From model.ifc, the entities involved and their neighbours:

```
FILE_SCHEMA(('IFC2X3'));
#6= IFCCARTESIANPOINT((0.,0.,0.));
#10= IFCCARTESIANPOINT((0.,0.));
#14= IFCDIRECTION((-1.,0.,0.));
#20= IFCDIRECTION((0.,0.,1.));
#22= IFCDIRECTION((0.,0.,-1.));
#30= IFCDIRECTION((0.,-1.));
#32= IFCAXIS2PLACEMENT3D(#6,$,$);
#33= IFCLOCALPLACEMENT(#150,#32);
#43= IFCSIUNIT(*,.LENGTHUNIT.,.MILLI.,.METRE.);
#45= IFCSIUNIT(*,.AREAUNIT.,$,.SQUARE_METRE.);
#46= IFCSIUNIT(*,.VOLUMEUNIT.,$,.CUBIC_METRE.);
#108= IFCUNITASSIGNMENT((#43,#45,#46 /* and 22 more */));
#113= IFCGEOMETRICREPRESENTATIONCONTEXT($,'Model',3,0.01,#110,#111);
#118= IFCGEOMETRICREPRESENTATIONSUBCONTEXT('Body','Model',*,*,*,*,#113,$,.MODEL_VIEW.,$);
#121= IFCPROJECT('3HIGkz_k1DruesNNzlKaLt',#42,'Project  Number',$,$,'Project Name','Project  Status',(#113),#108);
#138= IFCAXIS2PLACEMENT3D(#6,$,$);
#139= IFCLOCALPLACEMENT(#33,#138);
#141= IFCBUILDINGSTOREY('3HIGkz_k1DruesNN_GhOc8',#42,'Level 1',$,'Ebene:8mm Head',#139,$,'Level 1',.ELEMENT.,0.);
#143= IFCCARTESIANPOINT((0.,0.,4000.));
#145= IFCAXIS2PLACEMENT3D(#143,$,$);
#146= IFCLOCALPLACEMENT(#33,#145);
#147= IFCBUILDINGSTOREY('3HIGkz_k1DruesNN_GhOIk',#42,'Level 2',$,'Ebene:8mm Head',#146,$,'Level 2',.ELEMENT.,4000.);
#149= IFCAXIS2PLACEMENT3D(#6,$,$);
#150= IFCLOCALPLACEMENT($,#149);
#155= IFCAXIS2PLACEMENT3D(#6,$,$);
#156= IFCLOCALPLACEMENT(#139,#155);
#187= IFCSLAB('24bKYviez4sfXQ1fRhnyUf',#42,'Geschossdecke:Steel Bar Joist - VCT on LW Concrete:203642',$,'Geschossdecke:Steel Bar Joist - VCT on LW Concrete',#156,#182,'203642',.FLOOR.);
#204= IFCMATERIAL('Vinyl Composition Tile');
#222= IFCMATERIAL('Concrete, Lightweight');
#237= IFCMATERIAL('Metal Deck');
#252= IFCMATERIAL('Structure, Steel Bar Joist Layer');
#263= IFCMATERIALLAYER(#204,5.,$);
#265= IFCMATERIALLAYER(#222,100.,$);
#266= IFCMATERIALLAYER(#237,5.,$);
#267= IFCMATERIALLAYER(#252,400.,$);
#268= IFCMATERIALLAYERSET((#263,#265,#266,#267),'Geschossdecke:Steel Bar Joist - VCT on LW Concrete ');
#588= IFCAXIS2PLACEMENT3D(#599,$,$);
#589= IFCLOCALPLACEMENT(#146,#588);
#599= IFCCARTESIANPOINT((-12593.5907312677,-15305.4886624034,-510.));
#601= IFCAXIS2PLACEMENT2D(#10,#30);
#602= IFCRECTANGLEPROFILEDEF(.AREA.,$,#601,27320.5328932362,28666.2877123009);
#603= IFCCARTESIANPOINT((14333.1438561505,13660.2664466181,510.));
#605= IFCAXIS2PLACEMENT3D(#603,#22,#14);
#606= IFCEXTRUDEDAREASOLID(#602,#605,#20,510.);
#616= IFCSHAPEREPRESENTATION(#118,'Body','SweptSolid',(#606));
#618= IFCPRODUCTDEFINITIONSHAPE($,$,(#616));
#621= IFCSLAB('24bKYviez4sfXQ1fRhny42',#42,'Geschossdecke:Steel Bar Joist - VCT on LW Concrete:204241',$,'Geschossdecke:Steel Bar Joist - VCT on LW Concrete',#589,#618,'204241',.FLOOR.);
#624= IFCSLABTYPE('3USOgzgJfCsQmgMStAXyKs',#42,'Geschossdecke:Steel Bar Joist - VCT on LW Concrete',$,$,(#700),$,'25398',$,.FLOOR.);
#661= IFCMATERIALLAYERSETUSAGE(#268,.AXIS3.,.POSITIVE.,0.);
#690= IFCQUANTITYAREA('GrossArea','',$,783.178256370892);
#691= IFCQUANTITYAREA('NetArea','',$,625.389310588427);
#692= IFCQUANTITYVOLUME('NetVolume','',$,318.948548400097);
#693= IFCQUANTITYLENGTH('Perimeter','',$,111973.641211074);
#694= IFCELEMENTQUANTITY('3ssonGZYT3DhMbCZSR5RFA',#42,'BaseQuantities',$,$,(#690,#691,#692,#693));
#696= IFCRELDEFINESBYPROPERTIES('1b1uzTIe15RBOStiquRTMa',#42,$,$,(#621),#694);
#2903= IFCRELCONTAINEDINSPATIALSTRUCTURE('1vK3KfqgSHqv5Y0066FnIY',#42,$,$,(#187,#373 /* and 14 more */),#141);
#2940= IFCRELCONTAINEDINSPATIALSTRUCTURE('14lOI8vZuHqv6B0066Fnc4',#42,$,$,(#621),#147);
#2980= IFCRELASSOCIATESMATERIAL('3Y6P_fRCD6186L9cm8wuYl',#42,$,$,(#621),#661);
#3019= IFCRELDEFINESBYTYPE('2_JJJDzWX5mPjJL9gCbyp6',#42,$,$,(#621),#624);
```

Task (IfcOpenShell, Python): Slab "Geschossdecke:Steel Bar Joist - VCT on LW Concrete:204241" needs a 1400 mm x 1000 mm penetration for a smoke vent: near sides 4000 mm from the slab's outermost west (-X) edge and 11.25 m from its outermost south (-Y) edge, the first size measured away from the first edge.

```python
import numpy as np
import ifcopenshell
import ifcopenshell.api.feature
import ifcopenshell.api.geometry
import ifcopenshell.api.pset
import ifcopenshell.api.root
import ifcopenshell.geom
import ifcopenshell.util.element
import ifcopenshell.util.placement
import ifcopenshell.util.representation
import ifcopenshell.util.shape
import ifcopenshell.util.unit

model = ifcopenshell.open("model.ifc")
unit_scale = ifcopenshell.util.unit.calculate_unit_scale(model)
area_scale = ifcopenshell.util.unit.calculate_unit_scale(model, "AREAUNIT")
volume_scale = ifcopenshell.util.unit.calculate_unit_scale(model, "VOLUMEUNIT")
settings = ifcopenshell.geom.settings()


def volume(element):
    """Net volume in cubic metres, openings subtracted."""
    shape = ifcopenshell.geom.create_shape(settings, element)
    return ifcopenshell.util.shape.get_volume(shape.geometry)


slab = model.by_guid("24bKYviez4sfXQ1fRhny42")
before = volume(slab)

# Extent in the slab's own axes, in metres. The edges named are its -X and -Y sides.
slab_shape = ifcopenshell.geom.create_shape(settings, slab)
vertices = ifcopenshell.util.shape.get_vertices(slab_shape.geometry)
x_min, y_min, bottom = vertices.min(axis=0)
top = vertices[:, 2].max()

opening = ifcopenshell.api.root.create_entity(model, ifc_class="IfcOpeningElement", name="Smoke vent opening")
context = ifcopenshell.util.representation.get_context(model, "Model", "Body", "MODEL_VIEW")
width, depth = 1.4, 1
outline = [(0.0, 0.0), (width, 0.0), (width, depth), (0.0, depth), (0.0, 0.0)]
# Overshoot both faces by 50 mm so the cut is clean.
shape = ifcopenshell.api.geometry.add_slab_representation(
    model, context=context, depth=top - bottom + 0.1, polyline=outline
)
ifcopenshell.api.geometry.assign_representation(model, product=opening, representation=shape)

matrix = ifcopenshell.util.placement.get_local_placement(slab.ObjectPlacement)
matrix[:, 3] = matrix @ np.append(np.array([x_min + 4, y_min + 11.25, bottom - 0.05]) / unit_scale, 1.0)
ifcopenshell.api.geometry.edit_object_placement(model, product=opening, matrix=matrix, is_si=False)
ifcopenshell.api.feature.add_feature(model, feature=opening, element=slab)

after = volume(slab)

# Update the slab's stored quantities.
qto = model.by_id(ifcopenshell.util.element.get_pset(slab, "BaseQuantities", should_inherit=False)["id"])
ifcopenshell.api.pset.edit_qto(model, qto=qto, properties={
    "NetArea": after / (top - bottom) / area_scale,
    "NetVolume": after / volume_scale,
})

print(f"slab volume {before:.3f} -> {after:.3f} m3")

model.write("model_edited.ifc")
```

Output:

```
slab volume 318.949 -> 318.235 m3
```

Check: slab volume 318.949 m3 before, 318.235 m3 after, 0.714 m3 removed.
